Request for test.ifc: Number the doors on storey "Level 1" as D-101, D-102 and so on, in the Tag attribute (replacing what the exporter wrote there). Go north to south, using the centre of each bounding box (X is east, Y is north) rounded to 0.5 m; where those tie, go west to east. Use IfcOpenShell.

First a look at what the model holds.

```python
import ifcopenshell
import ifcopenshell.util.element
import ifcopenshell.util.placement

model = ifcopenshell.open("test.ifc")
print(model.schema)
storey = next(s for s in model.by_type("IfcBuildingStorey") if s.Name == "Level 1")
doors = [e for e in ifcopenshell.util.element.get_decomposition(storey) if e.is_a("IfcDoor")]
for e in sorted(doors, key=lambda e: e.id()):
    origin = ifcopenshell.util.placement.get_local_placement(e.ObjectPlacement)[:3, 3]
    print(e.id(), e.Tag, e.Name, origin.round(2) + 0.0, sep=" | ")
```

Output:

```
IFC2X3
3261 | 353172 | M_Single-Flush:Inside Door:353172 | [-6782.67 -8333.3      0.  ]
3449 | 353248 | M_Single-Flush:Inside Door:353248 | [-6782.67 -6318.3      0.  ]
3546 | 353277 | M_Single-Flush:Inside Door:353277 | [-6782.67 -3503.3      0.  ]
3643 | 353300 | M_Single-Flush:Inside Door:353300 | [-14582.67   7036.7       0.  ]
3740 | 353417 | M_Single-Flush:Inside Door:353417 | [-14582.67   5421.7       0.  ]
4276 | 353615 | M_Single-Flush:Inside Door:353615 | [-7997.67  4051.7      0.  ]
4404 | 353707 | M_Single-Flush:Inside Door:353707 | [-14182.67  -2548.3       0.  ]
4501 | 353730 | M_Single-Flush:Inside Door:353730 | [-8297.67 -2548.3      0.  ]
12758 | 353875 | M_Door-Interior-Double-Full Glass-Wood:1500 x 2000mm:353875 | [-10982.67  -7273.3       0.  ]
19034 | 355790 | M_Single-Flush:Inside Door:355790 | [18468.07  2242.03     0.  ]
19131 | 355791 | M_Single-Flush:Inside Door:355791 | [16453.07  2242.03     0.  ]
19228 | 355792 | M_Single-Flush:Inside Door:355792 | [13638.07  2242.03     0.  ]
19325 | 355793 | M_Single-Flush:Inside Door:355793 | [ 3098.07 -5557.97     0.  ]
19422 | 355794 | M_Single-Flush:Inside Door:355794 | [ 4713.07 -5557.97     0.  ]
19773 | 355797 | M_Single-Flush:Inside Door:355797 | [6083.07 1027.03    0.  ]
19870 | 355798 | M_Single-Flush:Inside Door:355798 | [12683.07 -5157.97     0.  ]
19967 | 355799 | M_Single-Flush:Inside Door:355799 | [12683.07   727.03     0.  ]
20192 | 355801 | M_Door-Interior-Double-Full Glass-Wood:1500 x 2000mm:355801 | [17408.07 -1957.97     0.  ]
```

```python
import ifcopenshell
import ifcopenshell.geom
import ifcopenshell.util.element
import ifcopenshell.util.shape

model = ifcopenshell.open("test.ifc")
settings = ifcopenshell.geom.settings()
settings.set("use-world-coords", True)


def centre(element):
    shape = ifcopenshell.geom.create_shape(settings, element)
    return ifcopenshell.util.shape.get_bbox_centroid(shape.geometry)


storey = next(s for s in model.by_type("IfcBuildingStorey") if s.Name == "Level 1")
doors = [e for e in ifcopenshell.util.element.get_decomposition(storey) if e.is_a("IfcDoor")]

# Insertion points can sit at a corner or the storey origin, so sort by the geometry (in metres).
centres = {e: centre(e) for e in doors}
doors.sort(key=lambda e: (-round(centres[e][1] / 0.5), centres[e][0]))

for i, e in enumerate(doors, start=1):
    number = f"D-1{i:02d}"
    e.Tag = number
    print(e.id(), number)

model.write("test-out.ifc")
```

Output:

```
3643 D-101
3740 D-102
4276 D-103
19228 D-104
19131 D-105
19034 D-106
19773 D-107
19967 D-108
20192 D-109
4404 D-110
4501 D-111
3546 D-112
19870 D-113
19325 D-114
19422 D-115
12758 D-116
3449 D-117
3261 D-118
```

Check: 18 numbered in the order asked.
